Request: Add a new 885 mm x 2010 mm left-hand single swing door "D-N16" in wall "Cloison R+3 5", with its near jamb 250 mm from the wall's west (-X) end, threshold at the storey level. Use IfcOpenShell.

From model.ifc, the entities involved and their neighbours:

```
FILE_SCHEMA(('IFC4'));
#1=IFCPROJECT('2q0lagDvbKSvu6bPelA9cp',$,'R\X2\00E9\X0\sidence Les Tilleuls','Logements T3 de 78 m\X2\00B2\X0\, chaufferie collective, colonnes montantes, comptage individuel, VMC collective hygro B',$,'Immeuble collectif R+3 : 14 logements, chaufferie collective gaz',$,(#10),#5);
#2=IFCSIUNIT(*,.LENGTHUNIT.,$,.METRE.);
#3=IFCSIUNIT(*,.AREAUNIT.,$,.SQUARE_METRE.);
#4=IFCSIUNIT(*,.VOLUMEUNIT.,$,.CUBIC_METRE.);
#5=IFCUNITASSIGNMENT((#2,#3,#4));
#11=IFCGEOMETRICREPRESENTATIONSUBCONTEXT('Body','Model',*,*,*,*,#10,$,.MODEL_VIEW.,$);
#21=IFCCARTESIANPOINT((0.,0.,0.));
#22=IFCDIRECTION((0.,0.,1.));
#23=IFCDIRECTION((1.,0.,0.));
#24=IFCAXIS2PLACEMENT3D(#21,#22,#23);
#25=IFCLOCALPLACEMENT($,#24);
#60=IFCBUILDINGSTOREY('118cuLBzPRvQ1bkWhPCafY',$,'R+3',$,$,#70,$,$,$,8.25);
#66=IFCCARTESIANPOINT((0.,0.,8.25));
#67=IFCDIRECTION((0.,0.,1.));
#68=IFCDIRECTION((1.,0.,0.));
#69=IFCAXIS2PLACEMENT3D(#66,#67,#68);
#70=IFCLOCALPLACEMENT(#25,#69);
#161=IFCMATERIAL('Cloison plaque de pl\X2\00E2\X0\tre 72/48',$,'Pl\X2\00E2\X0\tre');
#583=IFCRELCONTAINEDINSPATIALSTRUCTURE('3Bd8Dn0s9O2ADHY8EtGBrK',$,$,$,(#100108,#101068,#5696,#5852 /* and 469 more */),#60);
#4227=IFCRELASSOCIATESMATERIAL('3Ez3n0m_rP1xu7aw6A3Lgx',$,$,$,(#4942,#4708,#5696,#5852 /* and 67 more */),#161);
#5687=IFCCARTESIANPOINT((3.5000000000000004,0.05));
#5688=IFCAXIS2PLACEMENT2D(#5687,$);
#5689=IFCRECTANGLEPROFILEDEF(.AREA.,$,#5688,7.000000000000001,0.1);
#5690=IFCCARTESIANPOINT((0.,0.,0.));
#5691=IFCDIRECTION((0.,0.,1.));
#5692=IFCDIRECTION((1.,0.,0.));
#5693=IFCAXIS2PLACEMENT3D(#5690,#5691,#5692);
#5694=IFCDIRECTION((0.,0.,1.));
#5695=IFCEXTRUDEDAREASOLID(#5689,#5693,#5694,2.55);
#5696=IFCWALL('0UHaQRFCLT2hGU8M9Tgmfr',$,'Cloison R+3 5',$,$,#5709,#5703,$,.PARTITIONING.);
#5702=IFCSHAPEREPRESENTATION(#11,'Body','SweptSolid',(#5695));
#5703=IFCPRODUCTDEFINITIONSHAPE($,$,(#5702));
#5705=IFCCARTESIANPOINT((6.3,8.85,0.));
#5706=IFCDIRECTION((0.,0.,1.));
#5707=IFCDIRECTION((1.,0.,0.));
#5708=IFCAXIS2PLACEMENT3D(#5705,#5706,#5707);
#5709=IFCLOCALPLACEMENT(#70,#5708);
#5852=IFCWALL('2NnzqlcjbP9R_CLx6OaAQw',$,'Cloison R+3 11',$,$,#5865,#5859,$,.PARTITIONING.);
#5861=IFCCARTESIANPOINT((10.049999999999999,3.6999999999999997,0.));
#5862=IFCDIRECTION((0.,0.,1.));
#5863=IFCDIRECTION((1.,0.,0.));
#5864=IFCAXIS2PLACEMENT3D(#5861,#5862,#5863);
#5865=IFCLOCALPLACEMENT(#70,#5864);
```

```python
import numpy as np
import ifcopenshell
import ifcopenshell.api.feature
import ifcopenshell.api.geometry
import ifcopenshell.api.root
import ifcopenshell.api.spatial
import ifcopenshell.geom
import ifcopenshell.util.element
import ifcopenshell.util.placement
import ifcopenshell.util.representation
import ifcopenshell.util.shape
import ifcopenshell.util.unit

model = ifcopenshell.open("model.ifc")
unit_scale = ifcopenshell.util.unit.calculate_unit_scale(model)
settings = ifcopenshell.geom.settings()


def volume(element):
    """Net volume in cubic metres, openings subtracted."""
    shape = ifcopenshell.geom.create_shape(settings, element)
    return ifcopenshell.util.shape.get_volume(shape.geometry)


wall = model.by_guid("0UHaQRFCLT2hGU8M9Tgmfr")
storey = ifcopenshell.util.element.get_container(wall, ifc_class="IfcBuildingStorey")
context = ifcopenshell.util.representation.get_context(model, "Model", "Body", "MODEL_VIEW")
before = volume(wall)

width, height, from_end, sill = 0.885, 2.01, 0.25, 0.0  # metres

# The wall runs along its own X axis, and the end named is its -X end.
wall_shape = ifcopenshell.geom.create_shape(settings, wall)
x, y, z = ifcopenshell.util.shape.get_vertices(wall_shape.geometry).T
start = x.min() + from_end
face, thickness = float(y.min()), float(y.max() - y.min())
wall_matrix = ifcopenshell.util.placement.get_local_placement(wall.ObjectPlacement)
level = ifcopenshell.util.placement.get_local_placement(storey.ObjectPlacement)[2, 3]


def in_wall(x, y):
    """Placement at x, y metres in the wall's axes, at sill height."""
    matrix = wall_matrix.copy()
    matrix[:, 3] = wall_matrix @ np.array([x / unit_scale, y / unit_scale, 0.0, 1.0])
    matrix[2, 3] = level + sill / unit_scale
    return matrix


# Opening: a box that overshoots both wall faces by 50 mm.
opening = ifcopenshell.api.root.create_entity(model, ifc_class="IfcOpeningElement", predefined_type="OPENING")
box = ifcopenshell.api.geometry.add_wall_representation(
    model, context=context, length=width, height=height, thickness=thickness + 0.1
)
ifcopenshell.api.geometry.assign_representation(model, product=opening, representation=box)
ifcopenshell.api.geometry.edit_object_placement(model, product=opening, matrix=in_wall(start, face - 0.05), is_si=False)
ifcopenshell.api.feature.add_feature(model, feature=opening, element=wall)

door = ifcopenshell.api.root.create_entity(model, ifc_class="IfcDoor", name="D-N16", predefined_type="DOOR")
door.OverallWidth, door.OverallHeight = width / unit_scale, height / unit_scale
door.OperationType = "SINGLE_SWING_LEFT"
body = ifcopenshell.api.geometry.add_door_representation(
    model,
    context=context,
    overall_width=door.OverallWidth,
    overall_height=door.OverallHeight,
    operation_type="SINGLE_SWING_LEFT",
    lining_properties={"LiningDepth": thickness / unit_scale, "ThresholdDepth": thickness / unit_scale},
)
ifcopenshell.api.geometry.assign_representation(model, product=door, representation=body)
ifcopenshell.api.spatial.assign_container(model, products=[door], relating_structure=storey)
ifcopenshell.api.feature.add_filling(model, opening=opening, element=door)

# The lining spans the wall, so the door starts at the wall face.
ifcopenshell.api.geometry.edit_object_placement(model, product=door, matrix=in_wall(start, face), is_si=False)

after = volume(wall)

print(f"wall volume {before:.3f} -> {after:.3f} m3")

model.write("model_edited.ifc")
```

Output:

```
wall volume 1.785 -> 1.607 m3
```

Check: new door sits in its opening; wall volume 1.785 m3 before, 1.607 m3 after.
